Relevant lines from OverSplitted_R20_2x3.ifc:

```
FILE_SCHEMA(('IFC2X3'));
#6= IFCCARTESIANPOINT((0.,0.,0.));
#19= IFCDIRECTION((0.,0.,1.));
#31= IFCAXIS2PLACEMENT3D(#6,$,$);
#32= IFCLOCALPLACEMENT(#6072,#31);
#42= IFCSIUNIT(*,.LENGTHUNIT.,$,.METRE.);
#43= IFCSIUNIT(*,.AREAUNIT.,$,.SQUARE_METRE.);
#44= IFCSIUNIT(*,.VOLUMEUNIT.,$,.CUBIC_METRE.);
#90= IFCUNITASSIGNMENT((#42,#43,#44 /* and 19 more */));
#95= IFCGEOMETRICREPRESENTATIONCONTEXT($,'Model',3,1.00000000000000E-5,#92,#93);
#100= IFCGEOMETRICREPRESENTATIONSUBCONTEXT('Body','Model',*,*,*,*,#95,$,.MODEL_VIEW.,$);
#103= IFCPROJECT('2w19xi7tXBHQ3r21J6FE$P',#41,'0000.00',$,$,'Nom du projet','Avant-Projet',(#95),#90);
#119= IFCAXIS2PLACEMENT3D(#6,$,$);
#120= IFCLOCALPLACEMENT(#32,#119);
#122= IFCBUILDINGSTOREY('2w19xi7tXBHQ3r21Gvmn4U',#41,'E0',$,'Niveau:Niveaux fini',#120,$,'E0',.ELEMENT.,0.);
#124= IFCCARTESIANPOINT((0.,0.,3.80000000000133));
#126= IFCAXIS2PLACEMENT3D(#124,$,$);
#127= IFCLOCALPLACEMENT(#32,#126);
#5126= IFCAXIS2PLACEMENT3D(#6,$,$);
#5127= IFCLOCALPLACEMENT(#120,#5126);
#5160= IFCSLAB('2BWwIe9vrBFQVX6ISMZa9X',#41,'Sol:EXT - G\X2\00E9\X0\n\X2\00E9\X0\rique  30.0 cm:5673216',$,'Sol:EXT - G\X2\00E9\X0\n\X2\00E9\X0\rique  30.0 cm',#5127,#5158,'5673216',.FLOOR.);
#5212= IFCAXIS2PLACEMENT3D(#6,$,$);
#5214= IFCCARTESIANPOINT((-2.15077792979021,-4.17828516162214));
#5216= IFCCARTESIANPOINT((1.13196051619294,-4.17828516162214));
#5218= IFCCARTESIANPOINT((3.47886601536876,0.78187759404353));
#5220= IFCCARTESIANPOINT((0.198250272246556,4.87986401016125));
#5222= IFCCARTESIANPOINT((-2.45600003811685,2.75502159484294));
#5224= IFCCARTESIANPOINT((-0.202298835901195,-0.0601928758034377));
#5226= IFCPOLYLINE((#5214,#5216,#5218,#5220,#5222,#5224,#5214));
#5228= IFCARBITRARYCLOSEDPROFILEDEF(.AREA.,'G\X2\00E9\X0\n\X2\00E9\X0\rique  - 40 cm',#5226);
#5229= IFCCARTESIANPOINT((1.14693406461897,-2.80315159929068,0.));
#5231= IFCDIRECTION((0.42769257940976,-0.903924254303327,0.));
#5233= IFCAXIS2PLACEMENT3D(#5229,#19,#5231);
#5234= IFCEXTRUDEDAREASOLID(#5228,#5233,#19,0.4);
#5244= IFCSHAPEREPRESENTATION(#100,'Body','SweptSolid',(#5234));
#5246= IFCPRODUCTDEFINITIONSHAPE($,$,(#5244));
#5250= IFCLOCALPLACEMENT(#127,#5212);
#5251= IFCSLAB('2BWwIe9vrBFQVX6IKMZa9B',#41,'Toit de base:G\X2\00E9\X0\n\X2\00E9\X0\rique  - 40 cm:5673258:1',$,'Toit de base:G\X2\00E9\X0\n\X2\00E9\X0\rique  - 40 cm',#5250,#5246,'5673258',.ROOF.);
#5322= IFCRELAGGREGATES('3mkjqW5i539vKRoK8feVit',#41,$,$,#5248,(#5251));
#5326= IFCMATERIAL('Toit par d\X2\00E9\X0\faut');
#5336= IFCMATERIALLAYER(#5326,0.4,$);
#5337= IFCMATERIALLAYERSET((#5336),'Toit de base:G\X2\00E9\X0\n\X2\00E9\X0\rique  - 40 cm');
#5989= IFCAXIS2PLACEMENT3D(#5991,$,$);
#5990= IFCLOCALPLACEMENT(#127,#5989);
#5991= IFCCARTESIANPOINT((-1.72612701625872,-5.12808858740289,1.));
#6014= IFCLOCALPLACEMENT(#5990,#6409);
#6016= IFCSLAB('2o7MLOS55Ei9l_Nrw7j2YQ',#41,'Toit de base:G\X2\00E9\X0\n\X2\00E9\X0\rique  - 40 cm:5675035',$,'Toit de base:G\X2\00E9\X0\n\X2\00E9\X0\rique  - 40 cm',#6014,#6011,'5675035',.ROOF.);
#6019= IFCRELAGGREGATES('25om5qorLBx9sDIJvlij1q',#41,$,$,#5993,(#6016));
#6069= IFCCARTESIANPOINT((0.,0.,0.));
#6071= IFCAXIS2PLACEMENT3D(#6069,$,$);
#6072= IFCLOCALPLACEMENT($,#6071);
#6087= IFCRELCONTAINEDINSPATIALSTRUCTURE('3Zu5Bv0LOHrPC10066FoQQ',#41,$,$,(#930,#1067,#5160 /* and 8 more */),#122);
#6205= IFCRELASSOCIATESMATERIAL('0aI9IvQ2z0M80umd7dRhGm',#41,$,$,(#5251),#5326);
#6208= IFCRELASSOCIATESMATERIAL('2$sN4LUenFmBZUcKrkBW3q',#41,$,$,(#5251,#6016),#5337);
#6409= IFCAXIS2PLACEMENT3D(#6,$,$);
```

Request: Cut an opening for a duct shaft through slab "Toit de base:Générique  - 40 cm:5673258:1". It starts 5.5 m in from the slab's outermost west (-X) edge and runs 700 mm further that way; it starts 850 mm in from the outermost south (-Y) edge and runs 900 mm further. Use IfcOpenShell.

```python
import numpy as np
import ifcopenshell
import ifcopenshell.api.feature
import ifcopenshell.api.geometry
import ifcopenshell.api.root
import ifcopenshell.geom
import ifcopenshell.util.placement
import ifcopenshell.util.representation
import ifcopenshell.util.shape
import ifcopenshell.util.unit

model = ifcopenshell.open("OverSplitted_R20_2x3.ifc")
unit_scale = ifcopenshell.util.unit.calculate_unit_scale(model)
settings = ifcopenshell.geom.settings()


def volume(element):
    """Net volume in cubic metres, openings subtracted."""
    shape = ifcopenshell.geom.create_shape(settings, element)
    return ifcopenshell.util.shape.get_volume(shape.geometry)


slab = model.by_id(5251)
before = volume(slab)

# Extent in the slab's own axes, in metres. The edges named are its -X and -Y sides.
slab_shape = ifcopenshell.geom.create_shape(settings, slab)
vertices = ifcopenshell.util.shape.get_vertices(slab_shape.geometry)
x_min, y_min, bottom = vertices.min(axis=0)
top = vertices[:, 2].max()

opening = ifcopenshell.api.root.create_entity(model, ifc_class="IfcOpeningElement", name="Duct shaft opening")
context = ifcopenshell.util.representation.get_context(model, "Model", "Body", "MODEL_VIEW")
width, depth = 0.7, 0.9
outline = [(0.0, 0.0), (width, 0.0), (width, depth), (0.0, depth), (0.0, 0.0)]
# Overshoot both faces by 50 mm so the cut is clean.
shape = ifcopenshell.api.geometry.add_slab_representation(
    model, context=context, depth=top - bottom + 0.1, polyline=outline
)
ifcopenshell.api.geometry.assign_representation(model, product=opening, representation=shape)

matrix = ifcopenshell.util.placement.get_local_placement(slab.ObjectPlacement)
matrix[:, 3] = matrix @ np.append(np.array([x_min + 5.5, y_min + 0.85, bottom - 0.05]) / unit_scale, 1.0)
ifcopenshell.api.geometry.edit_object_placement(model, product=opening, matrix=matrix, is_si=False)
ifcopenshell.api.feature.add_feature(model, feature=opening, element=slab)

after = volume(slab)

print(f"slab volume {before:.3f} -> {after:.3f} m3")

model.write("OverSplitted_R20_2x3_v2.ifc")
```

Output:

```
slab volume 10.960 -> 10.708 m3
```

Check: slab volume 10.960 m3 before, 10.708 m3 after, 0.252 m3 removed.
